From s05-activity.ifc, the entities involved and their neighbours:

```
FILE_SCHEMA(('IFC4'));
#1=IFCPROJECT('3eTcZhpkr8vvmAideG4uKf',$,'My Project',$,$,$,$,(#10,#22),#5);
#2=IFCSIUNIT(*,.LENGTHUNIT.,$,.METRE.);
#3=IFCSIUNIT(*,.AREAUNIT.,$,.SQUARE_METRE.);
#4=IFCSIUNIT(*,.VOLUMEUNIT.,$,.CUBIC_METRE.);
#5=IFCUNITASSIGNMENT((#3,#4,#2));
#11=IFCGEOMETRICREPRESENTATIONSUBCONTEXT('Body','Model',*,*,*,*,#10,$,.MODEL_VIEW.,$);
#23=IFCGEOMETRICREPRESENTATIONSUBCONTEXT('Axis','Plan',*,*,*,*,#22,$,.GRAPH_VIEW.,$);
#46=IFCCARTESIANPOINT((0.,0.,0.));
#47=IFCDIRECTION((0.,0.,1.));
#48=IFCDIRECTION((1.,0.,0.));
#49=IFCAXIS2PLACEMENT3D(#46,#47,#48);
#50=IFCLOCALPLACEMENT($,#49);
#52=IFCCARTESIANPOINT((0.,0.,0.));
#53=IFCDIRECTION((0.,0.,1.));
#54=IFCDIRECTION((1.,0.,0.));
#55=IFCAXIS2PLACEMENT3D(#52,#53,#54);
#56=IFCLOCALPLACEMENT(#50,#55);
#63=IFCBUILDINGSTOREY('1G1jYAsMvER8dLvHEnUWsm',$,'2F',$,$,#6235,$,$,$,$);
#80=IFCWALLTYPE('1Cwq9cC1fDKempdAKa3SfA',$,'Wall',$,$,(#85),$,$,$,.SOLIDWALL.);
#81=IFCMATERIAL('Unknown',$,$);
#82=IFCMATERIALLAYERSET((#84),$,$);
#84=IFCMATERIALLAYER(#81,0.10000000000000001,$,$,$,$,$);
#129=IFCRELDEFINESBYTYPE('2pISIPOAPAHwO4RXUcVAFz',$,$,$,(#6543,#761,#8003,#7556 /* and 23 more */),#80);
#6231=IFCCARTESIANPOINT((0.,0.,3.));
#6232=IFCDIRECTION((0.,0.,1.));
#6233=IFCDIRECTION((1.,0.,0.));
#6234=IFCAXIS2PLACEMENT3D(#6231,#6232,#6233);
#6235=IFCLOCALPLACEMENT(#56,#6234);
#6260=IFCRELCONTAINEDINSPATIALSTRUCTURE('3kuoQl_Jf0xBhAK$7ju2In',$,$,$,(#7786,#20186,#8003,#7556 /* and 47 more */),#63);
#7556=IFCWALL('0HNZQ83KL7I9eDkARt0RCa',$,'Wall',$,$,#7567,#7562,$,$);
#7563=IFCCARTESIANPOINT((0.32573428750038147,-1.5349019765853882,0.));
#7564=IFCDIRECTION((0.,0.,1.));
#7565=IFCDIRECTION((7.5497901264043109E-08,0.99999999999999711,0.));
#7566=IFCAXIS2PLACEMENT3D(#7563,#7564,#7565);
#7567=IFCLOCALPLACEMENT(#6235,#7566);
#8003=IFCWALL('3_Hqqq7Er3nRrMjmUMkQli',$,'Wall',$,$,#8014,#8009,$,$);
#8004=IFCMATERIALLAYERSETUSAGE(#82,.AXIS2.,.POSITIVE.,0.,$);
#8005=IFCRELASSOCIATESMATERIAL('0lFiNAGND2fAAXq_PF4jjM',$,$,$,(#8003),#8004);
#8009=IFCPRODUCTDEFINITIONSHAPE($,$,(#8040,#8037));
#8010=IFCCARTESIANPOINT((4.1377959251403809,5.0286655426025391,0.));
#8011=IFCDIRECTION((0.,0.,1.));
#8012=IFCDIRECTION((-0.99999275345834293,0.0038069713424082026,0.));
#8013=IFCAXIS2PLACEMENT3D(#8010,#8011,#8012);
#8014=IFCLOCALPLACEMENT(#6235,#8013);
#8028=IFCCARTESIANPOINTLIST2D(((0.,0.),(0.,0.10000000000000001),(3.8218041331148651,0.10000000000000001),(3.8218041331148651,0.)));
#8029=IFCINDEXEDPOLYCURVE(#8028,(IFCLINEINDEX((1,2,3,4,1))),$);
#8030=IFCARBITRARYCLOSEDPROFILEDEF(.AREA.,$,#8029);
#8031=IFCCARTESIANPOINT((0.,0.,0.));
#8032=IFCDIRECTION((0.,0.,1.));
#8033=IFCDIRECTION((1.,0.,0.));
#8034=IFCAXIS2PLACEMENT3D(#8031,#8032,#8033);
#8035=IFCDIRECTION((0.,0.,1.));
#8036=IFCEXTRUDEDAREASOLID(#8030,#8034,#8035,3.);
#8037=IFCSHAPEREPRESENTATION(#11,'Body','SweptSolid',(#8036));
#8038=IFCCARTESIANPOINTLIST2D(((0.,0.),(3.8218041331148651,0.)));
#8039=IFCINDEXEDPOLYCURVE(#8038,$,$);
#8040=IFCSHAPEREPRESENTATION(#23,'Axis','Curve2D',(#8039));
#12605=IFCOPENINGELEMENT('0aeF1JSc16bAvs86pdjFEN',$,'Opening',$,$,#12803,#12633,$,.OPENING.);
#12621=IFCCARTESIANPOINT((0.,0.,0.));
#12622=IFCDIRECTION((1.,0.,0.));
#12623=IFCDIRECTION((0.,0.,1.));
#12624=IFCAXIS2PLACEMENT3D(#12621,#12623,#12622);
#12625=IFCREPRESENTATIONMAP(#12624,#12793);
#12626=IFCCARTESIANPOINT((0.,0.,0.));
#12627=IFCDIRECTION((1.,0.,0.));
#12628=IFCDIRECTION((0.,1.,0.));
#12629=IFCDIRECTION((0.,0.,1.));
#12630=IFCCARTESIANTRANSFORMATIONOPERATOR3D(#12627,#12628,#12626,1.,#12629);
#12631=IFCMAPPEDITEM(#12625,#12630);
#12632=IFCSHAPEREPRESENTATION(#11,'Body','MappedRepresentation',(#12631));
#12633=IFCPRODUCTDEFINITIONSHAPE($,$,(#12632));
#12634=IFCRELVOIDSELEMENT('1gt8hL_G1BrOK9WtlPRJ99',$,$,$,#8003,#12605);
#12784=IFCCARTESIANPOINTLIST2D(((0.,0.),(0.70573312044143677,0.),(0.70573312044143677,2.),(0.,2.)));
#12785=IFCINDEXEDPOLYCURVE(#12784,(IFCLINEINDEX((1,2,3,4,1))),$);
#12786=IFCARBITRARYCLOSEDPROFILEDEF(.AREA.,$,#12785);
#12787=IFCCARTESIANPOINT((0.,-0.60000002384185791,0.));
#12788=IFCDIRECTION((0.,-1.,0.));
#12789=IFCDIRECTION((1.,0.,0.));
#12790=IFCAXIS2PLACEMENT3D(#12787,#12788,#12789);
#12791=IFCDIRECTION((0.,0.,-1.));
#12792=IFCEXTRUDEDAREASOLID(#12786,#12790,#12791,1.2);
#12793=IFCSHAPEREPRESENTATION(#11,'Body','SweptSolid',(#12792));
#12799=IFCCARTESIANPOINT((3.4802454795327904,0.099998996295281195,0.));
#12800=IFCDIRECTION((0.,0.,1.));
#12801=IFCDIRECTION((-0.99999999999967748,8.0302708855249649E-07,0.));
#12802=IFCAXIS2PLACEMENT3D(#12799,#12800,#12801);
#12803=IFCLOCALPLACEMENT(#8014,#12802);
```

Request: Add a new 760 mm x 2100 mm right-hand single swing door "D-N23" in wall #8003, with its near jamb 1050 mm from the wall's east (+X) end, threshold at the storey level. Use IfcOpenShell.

```python
import numpy as np
import ifcopenshell
import ifcopenshell.api.feature
import ifcopenshell.api.geometry
import ifcopenshell.api.root
import ifcopenshell.api.spatial
import ifcopenshell.geom
import ifcopenshell.util.element
import ifcopenshell.util.placement
import ifcopenshell.util.representation
import ifcopenshell.util.shape
import ifcopenshell.util.unit

model = ifcopenshell.open("s05-activity.ifc")
unit_scale = ifcopenshell.util.unit.calculate_unit_scale(model)
settings = ifcopenshell.geom.settings()


def volume(element):
    """Net volume in cubic metres, openings subtracted."""
    shape = ifcopenshell.geom.create_shape(settings, element)
    return ifcopenshell.util.shape.get_volume(shape.geometry)


wall = model.by_id(8003)
storey = ifcopenshell.util.element.get_container(wall, ifc_class="IfcBuildingStorey")
context = ifcopenshell.util.representation.get_context(model, "Model", "Body", "MODEL_VIEW")
before = volume(wall)

width, height, from_end, sill = 0.76, 2.1, 1.05, 0.0  # metres

# The wall runs along its own X axis, and the end named is its -X end.
wall_shape = ifcopenshell.geom.create_shape(settings, wall)
x, y, z = ifcopenshell.util.shape.get_vertices(wall_shape.geometry).T
start = x.min() + from_end
face, thickness = float(y.min()), float(y.max() - y.min())
wall_matrix = ifcopenshell.util.placement.get_local_placement(wall.ObjectPlacement)
level = ifcopenshell.util.placement.get_local_placement(storey.ObjectPlacement)[2, 3]


def in_wall(x, y):
    """Placement at x, y metres in the wall's axes, at sill height."""
    matrix = wall_matrix.copy()
    matrix[:, 3] = wall_matrix @ np.array([x / unit_scale, y / unit_scale, 0.0, 1.0])
    matrix[2, 3] = level + sill / unit_scale
    return matrix


# Opening: a box that overshoots both wall faces by 50 mm.
opening = ifcopenshell.api.root.create_entity(model, ifc_class="IfcOpeningElement", predefined_type="OPENING")
box = ifcopenshell.api.geometry.add_wall_representation(
    model, context=context, length=width, height=height, thickness=thickness + 0.1
)
ifcopenshell.api.geometry.assign_representation(model, product=opening, representation=box)
ifcopenshell.api.geometry.edit_object_placement(model, product=opening, matrix=in_wall(start, face - 0.05), is_si=False)
ifcopenshell.api.feature.add_feature(model, feature=opening, element=wall)

door = ifcopenshell.api.root.create_entity(model, ifc_class="IfcDoor", name="D-N23", predefined_type="DOOR")
door.OverallWidth, door.OverallHeight = width / unit_scale, height / unit_scale
door.OperationType = "SINGLE_SWING_RIGHT"
body = ifcopenshell.api.geometry.add_door_representation(
    model,
    context=context,
    overall_width=door.OverallWidth,
    overall_height=door.OverallHeight,
    operation_type="SINGLE_SWING_RIGHT",
    lining_properties={"LiningDepth": thickness / unit_scale, "ThresholdDepth": thickness / unit_scale},
)
ifcopenshell.api.geometry.assign_representation(model, product=door, representation=body)
ifcopenshell.api.spatial.assign_container(model, products=[door], relating_structure=storey)
ifcopenshell.api.feature.add_filling(model, opening=opening, element=door)

# The lining spans the wall, so the door starts at the wall face.
ifcopenshell.api.geometry.edit_object_placement(model, product=door, matrix=in_wall(start, face), is_si=False)

after = volume(wall)

print(f"wall volume {before:.3f} -> {after:.3f} m3")

model.write("s05-activity-out.ifc")
```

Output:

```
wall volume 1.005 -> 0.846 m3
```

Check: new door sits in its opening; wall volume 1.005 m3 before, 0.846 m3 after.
